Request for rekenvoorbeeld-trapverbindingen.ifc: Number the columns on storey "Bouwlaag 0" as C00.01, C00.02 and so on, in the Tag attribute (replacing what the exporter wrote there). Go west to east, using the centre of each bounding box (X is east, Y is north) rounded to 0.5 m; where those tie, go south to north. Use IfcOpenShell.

First a look at what the model holds.

```python
import ifcopenshell
import ifcopenshell.util.element
import ifcopenshell.util.placement

model = ifcopenshell.open("rekenvoorbeeld-trapverbindingen.ifc")
print(model.schema)
storey = next(s for s in model.by_type("IfcBuildingStorey") if s.Name == "Bouwlaag 0")
columns = [e for e in ifcopenshell.util.element.get_decomposition(storey) if e.is_a("IfcColumn")]
for e in sorted(columns, key=lambda e: e.id()):
    origin = ifcopenshell.util.placement.get_local_placement(e.ObjectPlacement)[:3, 3]
    print(e.id(), e.Tag, e.Name, origin.round(2) + 0.0, sep=" | ")
```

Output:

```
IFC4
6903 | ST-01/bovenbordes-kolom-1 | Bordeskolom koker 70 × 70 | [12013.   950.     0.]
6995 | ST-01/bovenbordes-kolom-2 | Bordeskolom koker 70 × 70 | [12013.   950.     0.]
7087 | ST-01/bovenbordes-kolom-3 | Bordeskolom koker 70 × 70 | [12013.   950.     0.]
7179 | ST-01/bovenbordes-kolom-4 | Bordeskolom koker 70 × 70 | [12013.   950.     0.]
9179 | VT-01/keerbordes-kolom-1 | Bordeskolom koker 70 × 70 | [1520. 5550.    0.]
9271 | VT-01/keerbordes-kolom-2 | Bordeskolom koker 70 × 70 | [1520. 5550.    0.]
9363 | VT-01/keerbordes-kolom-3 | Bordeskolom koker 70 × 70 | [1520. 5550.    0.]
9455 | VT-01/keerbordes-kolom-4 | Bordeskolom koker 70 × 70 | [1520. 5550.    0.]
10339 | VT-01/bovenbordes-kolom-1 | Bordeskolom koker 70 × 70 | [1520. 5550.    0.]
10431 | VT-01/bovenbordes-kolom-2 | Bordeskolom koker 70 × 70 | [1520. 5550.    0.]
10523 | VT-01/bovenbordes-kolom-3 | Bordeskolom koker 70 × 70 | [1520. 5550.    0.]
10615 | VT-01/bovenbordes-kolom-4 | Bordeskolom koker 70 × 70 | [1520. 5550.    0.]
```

```python
import ifcopenshell
import ifcopenshell.geom
import ifcopenshell.util.element
import ifcopenshell.util.shape

model = ifcopenshell.open("rekenvoorbeeld-trapverbindingen.ifc")
settings = ifcopenshell.geom.settings()
settings.set("use-world-coords", True)


def centre(element):
    shape = ifcopenshell.geom.create_shape(settings, element)
    return ifcopenshell.util.shape.get_bbox_centroid(shape.geometry)


storey = next(s for s in model.by_type("IfcBuildingStorey") if s.Name == "Bouwlaag 0")
columns = [e for e in ifcopenshell.util.element.get_decomposition(storey) if e.is_a("IfcColumn")]

# Insertion points can sit at a corner or the storey origin, so sort by the geometry (in metres).
centres = {e: centre(e) for e in columns}
columns.sort(key=lambda e: (round(centres[e][0] / 0.5), centres[e][1]))

for i, e in enumerate(columns, start=1):
    number = f"C00.{i:02d}"
    e.Tag = number
    print(e.id(), number)

model.write("rekenvoorbeeld-trapverbindingen_rev.ifc")
```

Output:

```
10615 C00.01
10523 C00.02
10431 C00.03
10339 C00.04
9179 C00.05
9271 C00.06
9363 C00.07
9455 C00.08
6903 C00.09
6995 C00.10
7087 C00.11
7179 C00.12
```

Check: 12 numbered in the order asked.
